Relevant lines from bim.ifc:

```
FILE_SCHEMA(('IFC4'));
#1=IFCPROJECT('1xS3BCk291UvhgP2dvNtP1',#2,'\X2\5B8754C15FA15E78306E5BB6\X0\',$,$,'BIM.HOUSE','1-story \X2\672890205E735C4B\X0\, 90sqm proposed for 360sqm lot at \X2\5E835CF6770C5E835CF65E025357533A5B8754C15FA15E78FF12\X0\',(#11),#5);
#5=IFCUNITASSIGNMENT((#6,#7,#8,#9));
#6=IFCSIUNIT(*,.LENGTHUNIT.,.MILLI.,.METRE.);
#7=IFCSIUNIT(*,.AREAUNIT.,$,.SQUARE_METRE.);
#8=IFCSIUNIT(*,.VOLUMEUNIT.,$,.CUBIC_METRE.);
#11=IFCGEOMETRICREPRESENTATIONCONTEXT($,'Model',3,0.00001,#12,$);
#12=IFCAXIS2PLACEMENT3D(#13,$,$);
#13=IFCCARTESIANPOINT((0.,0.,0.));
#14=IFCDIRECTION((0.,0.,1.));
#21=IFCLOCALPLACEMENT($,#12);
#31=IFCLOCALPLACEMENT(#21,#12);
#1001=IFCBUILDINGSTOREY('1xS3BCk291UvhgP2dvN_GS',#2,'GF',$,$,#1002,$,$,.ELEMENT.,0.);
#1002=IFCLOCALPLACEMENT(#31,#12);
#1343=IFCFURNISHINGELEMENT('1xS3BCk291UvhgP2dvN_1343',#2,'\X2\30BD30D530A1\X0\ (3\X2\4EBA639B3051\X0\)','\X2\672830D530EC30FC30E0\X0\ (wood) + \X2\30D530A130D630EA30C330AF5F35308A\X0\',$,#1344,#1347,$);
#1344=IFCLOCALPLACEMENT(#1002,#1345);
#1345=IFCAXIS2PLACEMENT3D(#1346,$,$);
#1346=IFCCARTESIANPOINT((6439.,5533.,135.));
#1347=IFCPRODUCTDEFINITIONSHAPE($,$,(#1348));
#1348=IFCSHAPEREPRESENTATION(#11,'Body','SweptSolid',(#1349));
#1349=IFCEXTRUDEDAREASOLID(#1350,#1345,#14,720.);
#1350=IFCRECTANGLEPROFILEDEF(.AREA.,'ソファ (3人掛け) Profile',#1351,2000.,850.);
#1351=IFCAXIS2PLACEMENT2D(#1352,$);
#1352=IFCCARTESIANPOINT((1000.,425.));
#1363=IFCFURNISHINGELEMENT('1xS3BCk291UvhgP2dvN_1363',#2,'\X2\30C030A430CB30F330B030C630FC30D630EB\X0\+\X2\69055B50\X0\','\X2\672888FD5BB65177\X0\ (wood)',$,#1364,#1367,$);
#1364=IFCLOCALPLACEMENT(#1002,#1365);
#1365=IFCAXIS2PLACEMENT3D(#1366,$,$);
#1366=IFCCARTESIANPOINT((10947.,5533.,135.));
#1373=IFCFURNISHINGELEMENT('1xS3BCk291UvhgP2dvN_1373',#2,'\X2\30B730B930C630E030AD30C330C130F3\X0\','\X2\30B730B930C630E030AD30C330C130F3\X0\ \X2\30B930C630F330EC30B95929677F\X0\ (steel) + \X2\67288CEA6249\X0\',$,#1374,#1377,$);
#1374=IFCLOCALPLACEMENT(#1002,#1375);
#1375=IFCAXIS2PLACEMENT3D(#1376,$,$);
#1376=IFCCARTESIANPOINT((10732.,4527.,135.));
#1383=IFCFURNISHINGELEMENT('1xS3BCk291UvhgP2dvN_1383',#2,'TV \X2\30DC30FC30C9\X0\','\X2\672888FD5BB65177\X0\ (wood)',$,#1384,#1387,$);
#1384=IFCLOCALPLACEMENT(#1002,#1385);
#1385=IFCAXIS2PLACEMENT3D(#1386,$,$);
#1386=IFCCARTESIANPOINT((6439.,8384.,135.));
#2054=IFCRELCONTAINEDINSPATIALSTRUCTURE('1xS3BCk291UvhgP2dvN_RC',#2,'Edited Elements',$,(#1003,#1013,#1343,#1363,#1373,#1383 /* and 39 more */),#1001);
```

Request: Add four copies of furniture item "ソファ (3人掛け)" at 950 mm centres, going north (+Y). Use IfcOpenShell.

```python
import numpy as np
import ifcopenshell
import ifcopenshell.api.geometry
import ifcopenshell.api.root
import ifcopenshell.util.element
import ifcopenshell.util.placement
import ifcopenshell.util.unit

model = ifcopenshell.open("bim.ifc")
unit_scale = ifcopenshell.util.unit.calculate_unit_scale(model)


def reuse_history(source, copy):
    """copy_class also copies each property set's owner history, people and application; keep the originals."""
    for rel in copy.IsDefinedBy:
        if rel.is_a("IfcRelDefinesByProperties") and (history := rel.RelatingPropertyDefinition.OwnerHistory):
            rel.RelatingPropertyDefinition.OwnerHistory = source.OwnerHistory
            ifcopenshell.util.element.remove_deep2(model, history)


source = model.by_id(1343)
base = ifcopenshell.util.placement.get_local_placement(source.ObjectPlacement)
step = np.array([0.0, 1.0, 0.0]) * 0.95 / unit_scale

for i in range(1, 5):
    copy = ifcopenshell.api.root.copy_class(model, product=source)
    copy.Representation = ifcopenshell.util.element.copy_deep(
        model, source.Representation, exclude=["IfcGeometricRepresentationContext", "IfcRepresentationMap"]
    )
    reuse_history(source, copy)
    matrix = base.copy()
    matrix[:3, 3] += i * step
    print("added at", matrix[:3, 3].round(3) + 0.0)
    ifcopenshell.api.geometry.edit_object_placement(model, product=copy, matrix=matrix, is_si=False)

model.write("bim_v2.ifc")
```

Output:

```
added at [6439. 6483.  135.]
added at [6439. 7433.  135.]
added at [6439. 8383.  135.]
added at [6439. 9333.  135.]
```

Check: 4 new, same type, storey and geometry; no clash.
